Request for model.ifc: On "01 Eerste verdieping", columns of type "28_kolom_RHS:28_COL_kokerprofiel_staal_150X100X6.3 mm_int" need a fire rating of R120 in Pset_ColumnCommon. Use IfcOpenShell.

First a look at what the model holds.

```python
import ifcopenshell
import ifcopenshell.util.element

model = ifcopenshell.open("model.ifc")
print(model.schema)
storey = next(s for s in model.by_type("IfcBuildingStorey") if s.Name == "01 Eerste verdieping")
columns = [e for e in ifcopenshell.util.element.get_decomposition(storey) if e.is_a("IfcColumn")]
seen = {}
for e in columns:
    element_type = ifcopenshell.util.element.get_type(e)
    key = (element_type.Name if element_type != e and element_type else None, ifcopenshell.util.element.get_pset(e, "Pset_ColumnCommon", "FireRating"))
    seen[key] = seen.get(key, 0) + 1
for (name, value), count in sorted(seen.items(), key=str):
    print(count, "x", name, "|", value)
```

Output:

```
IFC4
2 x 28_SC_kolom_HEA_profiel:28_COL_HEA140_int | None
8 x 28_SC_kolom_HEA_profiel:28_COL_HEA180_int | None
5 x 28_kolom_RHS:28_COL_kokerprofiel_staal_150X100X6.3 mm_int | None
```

```python
import ifcopenshell
import ifcopenshell.api.pset
import ifcopenshell.util.element

model = ifcopenshell.open("model.ifc")

storey = next(s for s in model.by_type("IfcBuildingStorey") if s.Name == "01 Eerste verdieping")
columns = [e for e in ifcopenshell.util.element.get_decomposition(storey) if e.is_a("IfcColumn")]

count = 0
for e in columns:
    element_type = ifcopenshell.util.element.get_type(e)
    if element_type in (None, e) or element_type.Name != "28_kolom_RHS:28_COL_kokerprofiel_staal_150X100X6.3 mm_int":
        continue
    # add_pset returns the element's existing set when there is one.
    pset = ifcopenshell.api.pset.add_pset(model, product=e, name="Pset_ColumnCommon")
    ifcopenshell.api.pset.edit_pset(model, pset=pset, properties={"FireRating": "R120"})
    count += 1

print(count, "columns updated")

model.write("model_rev.ifc")
```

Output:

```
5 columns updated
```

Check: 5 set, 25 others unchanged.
